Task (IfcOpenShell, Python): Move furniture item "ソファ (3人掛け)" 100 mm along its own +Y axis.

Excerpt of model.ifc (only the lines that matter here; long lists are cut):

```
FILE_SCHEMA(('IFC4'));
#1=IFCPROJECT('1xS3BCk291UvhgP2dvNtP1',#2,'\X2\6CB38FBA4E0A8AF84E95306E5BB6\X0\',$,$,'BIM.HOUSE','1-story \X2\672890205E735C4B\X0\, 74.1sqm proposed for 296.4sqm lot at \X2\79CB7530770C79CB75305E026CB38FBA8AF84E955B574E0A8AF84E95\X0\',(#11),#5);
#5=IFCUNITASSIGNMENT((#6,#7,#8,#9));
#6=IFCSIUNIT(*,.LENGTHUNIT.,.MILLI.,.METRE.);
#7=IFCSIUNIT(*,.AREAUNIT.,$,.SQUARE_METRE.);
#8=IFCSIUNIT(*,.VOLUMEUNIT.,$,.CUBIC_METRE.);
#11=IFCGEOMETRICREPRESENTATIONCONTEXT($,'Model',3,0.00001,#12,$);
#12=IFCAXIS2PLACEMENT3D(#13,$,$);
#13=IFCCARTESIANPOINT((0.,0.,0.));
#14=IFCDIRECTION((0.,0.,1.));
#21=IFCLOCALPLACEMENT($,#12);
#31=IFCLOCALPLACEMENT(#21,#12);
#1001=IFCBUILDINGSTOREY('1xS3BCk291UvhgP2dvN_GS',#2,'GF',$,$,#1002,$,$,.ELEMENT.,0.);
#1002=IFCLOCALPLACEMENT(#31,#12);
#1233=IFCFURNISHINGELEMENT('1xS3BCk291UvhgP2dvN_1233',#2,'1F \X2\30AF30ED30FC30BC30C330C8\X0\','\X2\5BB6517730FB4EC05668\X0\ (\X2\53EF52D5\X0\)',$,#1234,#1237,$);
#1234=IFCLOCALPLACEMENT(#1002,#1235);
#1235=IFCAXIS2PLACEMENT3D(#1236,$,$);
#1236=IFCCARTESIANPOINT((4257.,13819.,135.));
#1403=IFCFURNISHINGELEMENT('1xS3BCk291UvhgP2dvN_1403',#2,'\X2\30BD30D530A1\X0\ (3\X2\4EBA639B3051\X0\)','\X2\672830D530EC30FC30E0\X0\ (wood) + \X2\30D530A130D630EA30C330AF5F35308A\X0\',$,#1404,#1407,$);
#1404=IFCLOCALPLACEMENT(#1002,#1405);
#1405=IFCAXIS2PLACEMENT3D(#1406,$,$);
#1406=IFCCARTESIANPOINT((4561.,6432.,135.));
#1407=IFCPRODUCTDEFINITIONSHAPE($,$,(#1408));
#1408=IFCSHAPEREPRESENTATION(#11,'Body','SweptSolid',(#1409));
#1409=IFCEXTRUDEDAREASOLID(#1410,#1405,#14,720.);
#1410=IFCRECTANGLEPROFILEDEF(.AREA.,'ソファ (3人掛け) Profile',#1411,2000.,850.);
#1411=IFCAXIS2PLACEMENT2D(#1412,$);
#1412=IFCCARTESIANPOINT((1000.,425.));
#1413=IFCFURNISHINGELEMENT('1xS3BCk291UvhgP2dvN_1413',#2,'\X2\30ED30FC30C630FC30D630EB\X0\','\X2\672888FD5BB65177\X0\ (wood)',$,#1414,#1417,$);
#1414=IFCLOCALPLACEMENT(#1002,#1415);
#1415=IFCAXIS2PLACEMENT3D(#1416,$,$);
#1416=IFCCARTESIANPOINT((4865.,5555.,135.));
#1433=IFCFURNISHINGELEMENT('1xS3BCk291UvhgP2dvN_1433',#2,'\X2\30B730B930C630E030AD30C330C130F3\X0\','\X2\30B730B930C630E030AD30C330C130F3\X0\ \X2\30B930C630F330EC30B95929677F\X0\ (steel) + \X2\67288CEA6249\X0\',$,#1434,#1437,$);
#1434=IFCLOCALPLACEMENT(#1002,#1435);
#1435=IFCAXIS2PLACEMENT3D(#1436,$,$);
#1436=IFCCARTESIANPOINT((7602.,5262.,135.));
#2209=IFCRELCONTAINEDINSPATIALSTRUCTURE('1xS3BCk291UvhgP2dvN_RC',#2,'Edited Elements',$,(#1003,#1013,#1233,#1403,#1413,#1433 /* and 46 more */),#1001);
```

```python
import ifcopenshell
import ifcopenshell.api.geometry
import ifcopenshell.util.placement

model = ifcopenshell.open("model.ifc")

item = model.by_guid("1xS3BCk291UvhgP2dvN_1403")
matrix = ifcopenshell.util.placement.get_local_placement(item.ObjectPlacement)
matrix[:3, 3] += matrix[:3, 1] * 100.0
ifcopenshell.api.geometry.edit_object_placement(model, product=item, matrix=matrix, is_si=False)

print(ifcopenshell.util.placement.get_local_placement(item.ObjectPlacement).round(3) + 0.0)

model.write("model_v2.ifc")
```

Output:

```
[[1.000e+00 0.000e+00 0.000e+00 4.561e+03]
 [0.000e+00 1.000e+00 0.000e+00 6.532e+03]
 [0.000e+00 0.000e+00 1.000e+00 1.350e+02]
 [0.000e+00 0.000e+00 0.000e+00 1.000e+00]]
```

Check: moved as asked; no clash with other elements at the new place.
